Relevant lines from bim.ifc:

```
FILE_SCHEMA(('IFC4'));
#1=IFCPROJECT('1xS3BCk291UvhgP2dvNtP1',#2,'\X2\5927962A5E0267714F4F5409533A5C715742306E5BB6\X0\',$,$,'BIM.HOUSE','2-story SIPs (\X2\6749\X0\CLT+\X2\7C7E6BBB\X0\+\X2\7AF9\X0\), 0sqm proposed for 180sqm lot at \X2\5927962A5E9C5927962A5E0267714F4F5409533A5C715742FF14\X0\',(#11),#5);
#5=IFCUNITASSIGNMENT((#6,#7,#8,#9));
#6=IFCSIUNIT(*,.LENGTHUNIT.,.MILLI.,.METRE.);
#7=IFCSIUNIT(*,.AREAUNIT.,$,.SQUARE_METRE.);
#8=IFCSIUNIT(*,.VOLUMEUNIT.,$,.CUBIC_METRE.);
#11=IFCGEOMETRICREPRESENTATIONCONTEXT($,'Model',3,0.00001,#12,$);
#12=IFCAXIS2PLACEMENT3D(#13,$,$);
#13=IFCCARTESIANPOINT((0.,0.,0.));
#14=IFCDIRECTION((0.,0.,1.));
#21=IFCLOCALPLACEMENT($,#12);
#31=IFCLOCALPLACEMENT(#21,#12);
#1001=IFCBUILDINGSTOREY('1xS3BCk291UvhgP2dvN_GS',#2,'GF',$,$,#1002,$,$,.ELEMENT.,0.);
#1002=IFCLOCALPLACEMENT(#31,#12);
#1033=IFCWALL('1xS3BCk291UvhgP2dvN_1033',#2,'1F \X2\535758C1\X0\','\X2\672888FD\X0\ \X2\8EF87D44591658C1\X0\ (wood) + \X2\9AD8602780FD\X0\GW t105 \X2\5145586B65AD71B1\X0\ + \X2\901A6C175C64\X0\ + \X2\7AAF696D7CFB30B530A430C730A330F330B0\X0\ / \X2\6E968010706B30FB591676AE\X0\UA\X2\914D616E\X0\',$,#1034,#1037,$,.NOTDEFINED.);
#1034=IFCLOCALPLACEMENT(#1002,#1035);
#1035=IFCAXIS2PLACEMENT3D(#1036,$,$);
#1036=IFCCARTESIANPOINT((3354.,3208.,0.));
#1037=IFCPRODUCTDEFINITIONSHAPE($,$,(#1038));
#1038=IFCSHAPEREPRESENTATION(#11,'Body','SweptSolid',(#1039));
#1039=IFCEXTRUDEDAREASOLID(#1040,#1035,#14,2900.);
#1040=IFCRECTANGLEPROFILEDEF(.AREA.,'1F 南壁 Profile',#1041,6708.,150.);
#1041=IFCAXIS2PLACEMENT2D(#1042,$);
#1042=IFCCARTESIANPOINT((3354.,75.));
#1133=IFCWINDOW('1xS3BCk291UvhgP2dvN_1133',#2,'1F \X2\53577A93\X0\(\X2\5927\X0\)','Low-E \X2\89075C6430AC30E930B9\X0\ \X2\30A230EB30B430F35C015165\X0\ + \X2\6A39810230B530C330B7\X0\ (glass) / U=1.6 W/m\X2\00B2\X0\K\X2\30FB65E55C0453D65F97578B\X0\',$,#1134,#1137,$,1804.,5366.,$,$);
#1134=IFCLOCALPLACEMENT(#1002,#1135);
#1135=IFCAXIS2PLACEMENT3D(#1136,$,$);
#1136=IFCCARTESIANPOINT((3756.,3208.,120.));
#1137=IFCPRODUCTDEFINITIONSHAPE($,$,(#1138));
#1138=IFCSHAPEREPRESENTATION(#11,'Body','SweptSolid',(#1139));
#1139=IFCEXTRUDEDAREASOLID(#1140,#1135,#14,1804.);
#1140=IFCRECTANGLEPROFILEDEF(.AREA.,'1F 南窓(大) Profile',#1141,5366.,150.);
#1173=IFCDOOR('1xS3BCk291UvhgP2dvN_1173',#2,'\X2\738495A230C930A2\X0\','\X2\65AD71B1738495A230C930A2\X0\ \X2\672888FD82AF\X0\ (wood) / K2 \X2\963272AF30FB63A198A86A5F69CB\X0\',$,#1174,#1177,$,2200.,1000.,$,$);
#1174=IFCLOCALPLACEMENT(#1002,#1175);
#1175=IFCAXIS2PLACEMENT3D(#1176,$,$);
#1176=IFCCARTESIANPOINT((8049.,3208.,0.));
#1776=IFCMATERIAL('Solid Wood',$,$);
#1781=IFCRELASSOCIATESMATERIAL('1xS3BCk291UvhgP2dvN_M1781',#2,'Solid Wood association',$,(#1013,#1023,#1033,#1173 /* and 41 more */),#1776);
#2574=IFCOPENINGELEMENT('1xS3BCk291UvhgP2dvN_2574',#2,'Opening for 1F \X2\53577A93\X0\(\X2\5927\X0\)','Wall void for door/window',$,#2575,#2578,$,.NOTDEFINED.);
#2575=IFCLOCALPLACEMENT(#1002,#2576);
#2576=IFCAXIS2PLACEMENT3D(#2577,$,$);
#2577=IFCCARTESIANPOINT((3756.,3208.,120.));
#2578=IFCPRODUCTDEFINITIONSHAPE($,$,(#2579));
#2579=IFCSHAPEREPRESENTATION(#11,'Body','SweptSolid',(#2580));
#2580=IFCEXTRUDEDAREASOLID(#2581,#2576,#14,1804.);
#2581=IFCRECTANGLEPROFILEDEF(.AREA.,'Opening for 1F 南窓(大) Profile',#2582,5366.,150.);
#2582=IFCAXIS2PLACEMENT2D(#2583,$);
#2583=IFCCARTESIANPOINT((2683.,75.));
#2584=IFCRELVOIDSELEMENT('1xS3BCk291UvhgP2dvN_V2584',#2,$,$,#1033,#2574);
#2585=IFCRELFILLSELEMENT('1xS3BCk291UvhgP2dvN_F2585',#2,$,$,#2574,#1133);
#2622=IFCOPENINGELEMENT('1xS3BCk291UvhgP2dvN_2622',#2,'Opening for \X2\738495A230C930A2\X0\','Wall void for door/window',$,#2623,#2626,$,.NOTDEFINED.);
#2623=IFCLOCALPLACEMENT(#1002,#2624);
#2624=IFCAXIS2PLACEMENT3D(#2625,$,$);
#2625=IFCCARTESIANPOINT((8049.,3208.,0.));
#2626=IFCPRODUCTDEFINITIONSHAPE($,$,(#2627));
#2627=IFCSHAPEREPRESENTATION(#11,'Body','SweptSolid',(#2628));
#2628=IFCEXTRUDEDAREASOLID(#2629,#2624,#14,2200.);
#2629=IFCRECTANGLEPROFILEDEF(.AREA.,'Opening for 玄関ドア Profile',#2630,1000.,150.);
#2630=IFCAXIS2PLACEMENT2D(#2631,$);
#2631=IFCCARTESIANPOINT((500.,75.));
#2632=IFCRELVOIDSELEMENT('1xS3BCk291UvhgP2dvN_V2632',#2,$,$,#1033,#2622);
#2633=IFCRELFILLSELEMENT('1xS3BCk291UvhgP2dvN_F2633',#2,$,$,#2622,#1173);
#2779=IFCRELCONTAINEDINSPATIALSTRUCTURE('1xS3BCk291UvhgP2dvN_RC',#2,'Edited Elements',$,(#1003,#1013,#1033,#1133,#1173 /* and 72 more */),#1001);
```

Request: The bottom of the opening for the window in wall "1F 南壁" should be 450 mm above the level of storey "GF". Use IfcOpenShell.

```python
import numpy as np
import ifcopenshell
import ifcopenshell.api.geometry
import ifcopenshell.geom
import ifcopenshell.util.element
import ifcopenshell.util.placement
import ifcopenshell.util.shape
import ifcopenshell.util.unit

model = ifcopenshell.open("bim.ifc")
unit_scale = ifcopenshell.util.unit.calculate_unit_scale(model)

window = model.by_guid("1xS3BCk291UvhgP2dvN_1133")
opening = window.FillsVoids[0].RelatingOpeningElement
storey = ifcopenshell.util.element.get_container(window, ifc_class="IfcBuildingStorey")
level = ifcopenshell.util.placement.get_local_placement(storey.ObjectPlacement)[2, 3]

# The opening's origin need not be at the sill, so measure its lowest point.
shape = ifcopenshell.geom.create_shape(ifcopenshell.geom.settings(), opening)
bottom = ifcopenshell.util.shape.get_shape_bottom_elevation(shape, shape.geometry) / unit_scale
dz = level + 450.0 - bottom

shift = np.array([0.0, 0.0, dz])
# The window is not placed relative to its opening, so move both.
for product in (opening, window):
    matrix = ifcopenshell.util.placement.get_local_placement(product.ObjectPlacement)
    matrix[:3, 3] += shift
    ifcopenshell.api.geometry.edit_object_placement(model, product=product, matrix=matrix, is_si=False)

print(f"moved by {dz * unit_scale:+.3f} m")

model.write("bim-out.ifc")
```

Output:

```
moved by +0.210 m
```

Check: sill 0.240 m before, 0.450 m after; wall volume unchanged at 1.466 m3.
